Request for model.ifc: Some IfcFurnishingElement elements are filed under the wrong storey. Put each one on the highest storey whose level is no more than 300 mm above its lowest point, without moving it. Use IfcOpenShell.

First a look at what the model holds.

```python
import ifcopenshell
import ifcopenshell.util.element
import ifcopenshell.util.placement

model = ifcopenshell.open("model.ifc")
print(model.schema)
for storey in model.by_type("IfcBuildingStorey"):
    level = ifcopenshell.util.placement.get_storey_elevation(storey)
    count = sum(e.is_a("IfcFurnishingElement") for e in ifcopenshell.util.element.get_contained(storey))
    print(storey.id(), storey.Name, round(level, 3), count, sep=" | ")
```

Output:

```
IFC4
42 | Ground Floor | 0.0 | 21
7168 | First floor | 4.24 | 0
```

```python
import ifcopenshell
import ifcopenshell.api.spatial
import ifcopenshell.geom
import ifcopenshell.util.element
import ifcopenshell.util.placement
import ifcopenshell.util.shape
import ifcopenshell.util.unit

model = ifcopenshell.open("model.ifc")
unit_scale = ifcopenshell.util.unit.calculate_unit_scale(model)
settings = ifcopenshell.geom.settings()

levels = sorted(
    ((ifcopenshell.util.placement.get_storey_elevation(s) * unit_scale, s) for s in model.by_type("IfcBuildingStorey")),
    key=lambda pair: pair[0],
)

for e in model.by_type("IfcFurnishingElement"):
    current = e.ContainedInStructure[0].RelatingStructure if e.ContainedInStructure else None
    if current is None or not current.is_a("IfcBuildingStorey"):
        continue
    shape = ifcopenshell.geom.create_shape(settings, e)
    bottom = ifcopenshell.util.shape.get_shape_bottom_elevation(shape, shape.geometry)
    below = [s for level, s in levels if level <= bottom + 0.3]
    storey = below[-1] if below else levels[0][1]
    if storey != current:
        # assign_container keeps the world position.
        ifcopenshell.api.spatial.assign_container(model, products=[e], relating_structure=storey)
        print(e.id(), current.Name, "->", storey.Name)

model.write("model_edited.ifc")
```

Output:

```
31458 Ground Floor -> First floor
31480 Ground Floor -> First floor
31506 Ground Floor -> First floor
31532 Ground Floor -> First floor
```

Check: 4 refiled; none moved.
